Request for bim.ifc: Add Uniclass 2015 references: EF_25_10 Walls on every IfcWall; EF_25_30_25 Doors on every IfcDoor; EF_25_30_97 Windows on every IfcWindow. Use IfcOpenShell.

First a look at what the model holds.

```python
import ifcopenshell

model = ifcopenshell.open("bim.ifc")
print(model.schema)
print("classifications:", [c.Name for c in model.by_type("IfcClassification")])
for ifc_class in ("IfcDoor", "IfcRoof", "IfcStair", "IfcWall", "IfcWindow"):
    print(ifc_class, len(model.by_type(ifc_class)))
```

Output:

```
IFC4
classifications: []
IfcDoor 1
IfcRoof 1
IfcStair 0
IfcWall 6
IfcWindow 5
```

```python
import ifcopenshell
import ifcopenshell.api.classification

model = ifcopenshell.open("bim.ifc")

system = ifcopenshell.api.classification.add_classification(model, classification="Uniclass 2015")

codes = {
    "IfcWall": ("EF_25_10", "Walls"),
    "IfcDoor": ("EF_25_30_25", "Doors"),
    "IfcWindow": ("EF_25_30_97", "Windows"),
}
for ifc_class, (code, name) in codes.items():
    products = model.by_type(ifc_class)
    ifcopenshell.api.classification.add_reference(
        model, products=products, classification=system, identification=code, name=name
    )
    print(code, len(products))

model.write("bim_rev.ifc")
```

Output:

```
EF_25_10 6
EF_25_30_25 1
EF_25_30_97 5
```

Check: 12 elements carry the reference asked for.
